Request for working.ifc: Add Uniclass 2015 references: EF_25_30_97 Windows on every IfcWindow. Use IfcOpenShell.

First a look at what the model holds.

```python
import ifcopenshell

model = ifcopenshell.open("working.ifc")
print(model.schema)
print("classifications:", [c.Name for c in model.by_type("IfcClassification")])
for ifc_class in ("IfcDoor", "IfcRoof", "IfcStair", "IfcWall", "IfcWindow"):
    print(ifc_class, len(model.by_type(ifc_class)))
```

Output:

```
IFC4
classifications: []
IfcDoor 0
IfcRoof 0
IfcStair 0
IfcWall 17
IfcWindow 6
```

```python
import ifcopenshell
import ifcopenshell.api.classification

model = ifcopenshell.open("working.ifc")

system = ifcopenshell.api.classification.add_classification(model, classification="Uniclass 2015")

codes = {
    "IfcWindow": ("EF_25_30_97", "Windows"),
}
for ifc_class, (code, name) in codes.items():
    products = model.by_type(ifc_class)
    ifcopenshell.api.classification.add_reference(
        model, products=products, classification=system, identification=code, name=name
    )
    print(code, len(products))

model.write("working_v2.ifc")
```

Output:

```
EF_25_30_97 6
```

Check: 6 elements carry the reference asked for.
